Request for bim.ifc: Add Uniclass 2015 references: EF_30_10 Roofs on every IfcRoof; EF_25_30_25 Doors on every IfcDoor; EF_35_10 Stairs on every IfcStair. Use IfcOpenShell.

First a look at what the model holds.

```python
import ifcopenshell

model = ifcopenshell.open("bim.ifc")
print(model.schema)
print("classifications:", [c.Name for c in model.by_type("IfcClassification")])
for ifc_class in ("IfcDoor", "IfcRoof", "IfcStair", "IfcWall", "IfcWindow"):
    print(ifc_class, len(model.by_type(ifc_class)))
```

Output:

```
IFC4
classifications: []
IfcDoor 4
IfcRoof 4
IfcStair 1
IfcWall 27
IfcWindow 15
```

```python
import ifcopenshell
import ifcopenshell.api.classification

model = ifcopenshell.open("bim.ifc")

system = ifcopenshell.api.classification.add_classification(model, classification="Uniclass 2015")

codes = {
    "IfcRoof": ("EF_30_10", "Roofs"),
    "IfcDoor": ("EF_25_30_25", "Doors"),
    "IfcStair": ("EF_35_10", "Stairs"),
}
for ifc_class, (code, name) in codes.items():
    products = model.by_type(ifc_class)
    ifcopenshell.api.classification.add_reference(
        model, products=products, classification=system, identification=code, name=name
    )
    print(code, len(products))

model.write("bim_v2.ifc")
```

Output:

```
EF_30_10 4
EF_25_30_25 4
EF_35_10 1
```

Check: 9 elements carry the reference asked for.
